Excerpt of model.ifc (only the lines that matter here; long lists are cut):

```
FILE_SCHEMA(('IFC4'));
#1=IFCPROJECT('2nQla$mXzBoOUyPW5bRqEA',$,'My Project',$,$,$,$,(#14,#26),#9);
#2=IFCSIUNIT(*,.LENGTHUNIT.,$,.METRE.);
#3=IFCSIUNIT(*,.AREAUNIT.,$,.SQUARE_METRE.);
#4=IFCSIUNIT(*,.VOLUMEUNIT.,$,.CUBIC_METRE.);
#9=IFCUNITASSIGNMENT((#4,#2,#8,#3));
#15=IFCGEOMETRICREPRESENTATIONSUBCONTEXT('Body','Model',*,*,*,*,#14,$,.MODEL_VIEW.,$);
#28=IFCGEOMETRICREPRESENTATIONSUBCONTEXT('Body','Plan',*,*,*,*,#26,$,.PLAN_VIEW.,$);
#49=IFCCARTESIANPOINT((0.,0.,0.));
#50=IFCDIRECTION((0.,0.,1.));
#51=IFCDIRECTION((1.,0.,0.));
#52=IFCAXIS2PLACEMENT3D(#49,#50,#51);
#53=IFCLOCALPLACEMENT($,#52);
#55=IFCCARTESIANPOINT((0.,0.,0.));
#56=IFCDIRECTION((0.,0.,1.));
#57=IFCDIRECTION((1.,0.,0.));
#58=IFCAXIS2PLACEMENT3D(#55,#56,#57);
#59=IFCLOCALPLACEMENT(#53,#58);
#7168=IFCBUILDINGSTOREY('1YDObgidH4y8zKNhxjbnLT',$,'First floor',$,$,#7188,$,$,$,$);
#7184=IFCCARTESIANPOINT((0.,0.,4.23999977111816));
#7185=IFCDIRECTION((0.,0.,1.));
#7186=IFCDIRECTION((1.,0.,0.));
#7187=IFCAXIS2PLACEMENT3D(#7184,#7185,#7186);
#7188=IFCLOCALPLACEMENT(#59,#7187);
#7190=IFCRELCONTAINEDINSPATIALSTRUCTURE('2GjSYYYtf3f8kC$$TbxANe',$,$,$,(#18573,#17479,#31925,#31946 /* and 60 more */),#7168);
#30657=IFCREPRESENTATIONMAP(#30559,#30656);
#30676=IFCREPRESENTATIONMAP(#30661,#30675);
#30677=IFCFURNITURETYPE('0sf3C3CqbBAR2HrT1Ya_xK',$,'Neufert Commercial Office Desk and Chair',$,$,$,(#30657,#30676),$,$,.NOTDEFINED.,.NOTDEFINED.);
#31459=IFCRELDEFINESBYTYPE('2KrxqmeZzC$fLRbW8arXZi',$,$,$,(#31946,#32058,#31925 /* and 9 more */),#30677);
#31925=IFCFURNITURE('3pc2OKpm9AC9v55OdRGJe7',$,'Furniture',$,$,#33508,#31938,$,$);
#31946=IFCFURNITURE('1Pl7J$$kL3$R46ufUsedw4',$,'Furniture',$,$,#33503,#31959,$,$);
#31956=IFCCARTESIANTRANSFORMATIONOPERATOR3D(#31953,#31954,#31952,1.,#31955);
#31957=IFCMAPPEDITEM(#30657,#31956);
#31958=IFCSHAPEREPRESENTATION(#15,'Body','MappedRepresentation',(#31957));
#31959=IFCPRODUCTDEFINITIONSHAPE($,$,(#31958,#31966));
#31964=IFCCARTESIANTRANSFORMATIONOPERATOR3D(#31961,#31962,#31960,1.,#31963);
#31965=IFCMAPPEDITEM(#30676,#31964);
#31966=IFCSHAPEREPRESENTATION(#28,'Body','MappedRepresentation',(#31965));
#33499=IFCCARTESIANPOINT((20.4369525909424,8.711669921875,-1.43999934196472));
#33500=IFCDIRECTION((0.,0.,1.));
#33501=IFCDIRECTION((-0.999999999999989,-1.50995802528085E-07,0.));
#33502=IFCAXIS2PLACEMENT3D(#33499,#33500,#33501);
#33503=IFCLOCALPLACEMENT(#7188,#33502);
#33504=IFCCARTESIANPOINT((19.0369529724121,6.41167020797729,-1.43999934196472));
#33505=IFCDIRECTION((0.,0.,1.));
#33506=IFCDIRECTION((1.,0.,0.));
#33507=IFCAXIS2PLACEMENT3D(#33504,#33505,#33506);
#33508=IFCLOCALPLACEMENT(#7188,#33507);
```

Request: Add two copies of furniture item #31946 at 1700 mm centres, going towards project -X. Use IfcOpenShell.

```python
import numpy as np
import ifcopenshell
import ifcopenshell.api.geometry
import ifcopenshell.api.root
import ifcopenshell.util.element
import ifcopenshell.util.placement

model = ifcopenshell.open("model.ifc")

source = model.by_id(31946)
base = ifcopenshell.util.placement.get_local_placement(source.ObjectPlacement)
step = np.array([-1.0, 0.0, 0.0]) * 1.7

for i in range(1, 3):
    copy = ifcopenshell.api.root.copy_class(model, product=source)
    copy.Representation = ifcopenshell.util.element.copy_deep(
        model, source.Representation, exclude=["IfcGeometricRepresentationContext", "IfcRepresentationMap"]
    )
    matrix = base.copy()
    matrix[:3, 3] += i * step
    print("added at", matrix[:3, 3].round(3) + 0.0)
    ifcopenshell.api.geometry.edit_object_placement(model, product=copy, matrix=matrix, is_si=False)

model.write("model_updated.ifc")
```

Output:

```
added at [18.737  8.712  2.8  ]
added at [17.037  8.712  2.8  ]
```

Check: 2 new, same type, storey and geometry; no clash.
